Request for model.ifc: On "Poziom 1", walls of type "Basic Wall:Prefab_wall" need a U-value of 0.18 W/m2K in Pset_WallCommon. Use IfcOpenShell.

First a look at what the model holds.

```python
import ifcopenshell
import ifcopenshell.util.element

model = ifcopenshell.open("model.ifc")
print(model.schema)
storey = next(s for s in model.by_type("IfcBuildingStorey") if s.Name == "Poziom 1")
walls = [e for e in ifcopenshell.util.element.get_decomposition(storey) if e.is_a("IfcWall")]
seen = {}
for e in walls:
    element_type = ifcopenshell.util.element.get_type(e)
    key = (element_type.Name if element_type != e and element_type else None, ifcopenshell.util.element.get_pset(e, "Pset_WallCommon", "ThermalTransmittance"))
    seen[key] = seen.get(key, 0) + 1
for (name, value), count in sorted(seen.items(), key=str):
    print(count, "x", name, "|", value)
```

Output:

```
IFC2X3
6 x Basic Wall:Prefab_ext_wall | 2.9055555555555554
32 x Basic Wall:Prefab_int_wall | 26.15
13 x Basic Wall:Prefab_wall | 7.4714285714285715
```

```python
import ifcopenshell
import ifcopenshell.api.pset
import ifcopenshell.util.element

model = ifcopenshell.open("model.ifc")

storey = next(s for s in model.by_type("IfcBuildingStorey") if s.Name == "Poziom 1")
walls = [e for e in ifcopenshell.util.element.get_decomposition(storey) if e.is_a("IfcWall")]

count = 0
for e in walls:
    element_type = ifcopenshell.util.element.get_type(e)
    if element_type in (None, e) or element_type.Name != "Basic Wall:Prefab_wall":
        continue
    # add_pset returns the element's existing set when there is one.
    pset = ifcopenshell.api.pset.add_pset(model, product=e, name="Pset_WallCommon")
    ifcopenshell.api.pset.edit_pset(model, pset=pset, properties={"ThermalTransmittance": 0.18})
    count += 1

print(count, "walls updated")

model.write("model_edited.ifc")
```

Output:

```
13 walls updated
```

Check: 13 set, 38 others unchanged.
